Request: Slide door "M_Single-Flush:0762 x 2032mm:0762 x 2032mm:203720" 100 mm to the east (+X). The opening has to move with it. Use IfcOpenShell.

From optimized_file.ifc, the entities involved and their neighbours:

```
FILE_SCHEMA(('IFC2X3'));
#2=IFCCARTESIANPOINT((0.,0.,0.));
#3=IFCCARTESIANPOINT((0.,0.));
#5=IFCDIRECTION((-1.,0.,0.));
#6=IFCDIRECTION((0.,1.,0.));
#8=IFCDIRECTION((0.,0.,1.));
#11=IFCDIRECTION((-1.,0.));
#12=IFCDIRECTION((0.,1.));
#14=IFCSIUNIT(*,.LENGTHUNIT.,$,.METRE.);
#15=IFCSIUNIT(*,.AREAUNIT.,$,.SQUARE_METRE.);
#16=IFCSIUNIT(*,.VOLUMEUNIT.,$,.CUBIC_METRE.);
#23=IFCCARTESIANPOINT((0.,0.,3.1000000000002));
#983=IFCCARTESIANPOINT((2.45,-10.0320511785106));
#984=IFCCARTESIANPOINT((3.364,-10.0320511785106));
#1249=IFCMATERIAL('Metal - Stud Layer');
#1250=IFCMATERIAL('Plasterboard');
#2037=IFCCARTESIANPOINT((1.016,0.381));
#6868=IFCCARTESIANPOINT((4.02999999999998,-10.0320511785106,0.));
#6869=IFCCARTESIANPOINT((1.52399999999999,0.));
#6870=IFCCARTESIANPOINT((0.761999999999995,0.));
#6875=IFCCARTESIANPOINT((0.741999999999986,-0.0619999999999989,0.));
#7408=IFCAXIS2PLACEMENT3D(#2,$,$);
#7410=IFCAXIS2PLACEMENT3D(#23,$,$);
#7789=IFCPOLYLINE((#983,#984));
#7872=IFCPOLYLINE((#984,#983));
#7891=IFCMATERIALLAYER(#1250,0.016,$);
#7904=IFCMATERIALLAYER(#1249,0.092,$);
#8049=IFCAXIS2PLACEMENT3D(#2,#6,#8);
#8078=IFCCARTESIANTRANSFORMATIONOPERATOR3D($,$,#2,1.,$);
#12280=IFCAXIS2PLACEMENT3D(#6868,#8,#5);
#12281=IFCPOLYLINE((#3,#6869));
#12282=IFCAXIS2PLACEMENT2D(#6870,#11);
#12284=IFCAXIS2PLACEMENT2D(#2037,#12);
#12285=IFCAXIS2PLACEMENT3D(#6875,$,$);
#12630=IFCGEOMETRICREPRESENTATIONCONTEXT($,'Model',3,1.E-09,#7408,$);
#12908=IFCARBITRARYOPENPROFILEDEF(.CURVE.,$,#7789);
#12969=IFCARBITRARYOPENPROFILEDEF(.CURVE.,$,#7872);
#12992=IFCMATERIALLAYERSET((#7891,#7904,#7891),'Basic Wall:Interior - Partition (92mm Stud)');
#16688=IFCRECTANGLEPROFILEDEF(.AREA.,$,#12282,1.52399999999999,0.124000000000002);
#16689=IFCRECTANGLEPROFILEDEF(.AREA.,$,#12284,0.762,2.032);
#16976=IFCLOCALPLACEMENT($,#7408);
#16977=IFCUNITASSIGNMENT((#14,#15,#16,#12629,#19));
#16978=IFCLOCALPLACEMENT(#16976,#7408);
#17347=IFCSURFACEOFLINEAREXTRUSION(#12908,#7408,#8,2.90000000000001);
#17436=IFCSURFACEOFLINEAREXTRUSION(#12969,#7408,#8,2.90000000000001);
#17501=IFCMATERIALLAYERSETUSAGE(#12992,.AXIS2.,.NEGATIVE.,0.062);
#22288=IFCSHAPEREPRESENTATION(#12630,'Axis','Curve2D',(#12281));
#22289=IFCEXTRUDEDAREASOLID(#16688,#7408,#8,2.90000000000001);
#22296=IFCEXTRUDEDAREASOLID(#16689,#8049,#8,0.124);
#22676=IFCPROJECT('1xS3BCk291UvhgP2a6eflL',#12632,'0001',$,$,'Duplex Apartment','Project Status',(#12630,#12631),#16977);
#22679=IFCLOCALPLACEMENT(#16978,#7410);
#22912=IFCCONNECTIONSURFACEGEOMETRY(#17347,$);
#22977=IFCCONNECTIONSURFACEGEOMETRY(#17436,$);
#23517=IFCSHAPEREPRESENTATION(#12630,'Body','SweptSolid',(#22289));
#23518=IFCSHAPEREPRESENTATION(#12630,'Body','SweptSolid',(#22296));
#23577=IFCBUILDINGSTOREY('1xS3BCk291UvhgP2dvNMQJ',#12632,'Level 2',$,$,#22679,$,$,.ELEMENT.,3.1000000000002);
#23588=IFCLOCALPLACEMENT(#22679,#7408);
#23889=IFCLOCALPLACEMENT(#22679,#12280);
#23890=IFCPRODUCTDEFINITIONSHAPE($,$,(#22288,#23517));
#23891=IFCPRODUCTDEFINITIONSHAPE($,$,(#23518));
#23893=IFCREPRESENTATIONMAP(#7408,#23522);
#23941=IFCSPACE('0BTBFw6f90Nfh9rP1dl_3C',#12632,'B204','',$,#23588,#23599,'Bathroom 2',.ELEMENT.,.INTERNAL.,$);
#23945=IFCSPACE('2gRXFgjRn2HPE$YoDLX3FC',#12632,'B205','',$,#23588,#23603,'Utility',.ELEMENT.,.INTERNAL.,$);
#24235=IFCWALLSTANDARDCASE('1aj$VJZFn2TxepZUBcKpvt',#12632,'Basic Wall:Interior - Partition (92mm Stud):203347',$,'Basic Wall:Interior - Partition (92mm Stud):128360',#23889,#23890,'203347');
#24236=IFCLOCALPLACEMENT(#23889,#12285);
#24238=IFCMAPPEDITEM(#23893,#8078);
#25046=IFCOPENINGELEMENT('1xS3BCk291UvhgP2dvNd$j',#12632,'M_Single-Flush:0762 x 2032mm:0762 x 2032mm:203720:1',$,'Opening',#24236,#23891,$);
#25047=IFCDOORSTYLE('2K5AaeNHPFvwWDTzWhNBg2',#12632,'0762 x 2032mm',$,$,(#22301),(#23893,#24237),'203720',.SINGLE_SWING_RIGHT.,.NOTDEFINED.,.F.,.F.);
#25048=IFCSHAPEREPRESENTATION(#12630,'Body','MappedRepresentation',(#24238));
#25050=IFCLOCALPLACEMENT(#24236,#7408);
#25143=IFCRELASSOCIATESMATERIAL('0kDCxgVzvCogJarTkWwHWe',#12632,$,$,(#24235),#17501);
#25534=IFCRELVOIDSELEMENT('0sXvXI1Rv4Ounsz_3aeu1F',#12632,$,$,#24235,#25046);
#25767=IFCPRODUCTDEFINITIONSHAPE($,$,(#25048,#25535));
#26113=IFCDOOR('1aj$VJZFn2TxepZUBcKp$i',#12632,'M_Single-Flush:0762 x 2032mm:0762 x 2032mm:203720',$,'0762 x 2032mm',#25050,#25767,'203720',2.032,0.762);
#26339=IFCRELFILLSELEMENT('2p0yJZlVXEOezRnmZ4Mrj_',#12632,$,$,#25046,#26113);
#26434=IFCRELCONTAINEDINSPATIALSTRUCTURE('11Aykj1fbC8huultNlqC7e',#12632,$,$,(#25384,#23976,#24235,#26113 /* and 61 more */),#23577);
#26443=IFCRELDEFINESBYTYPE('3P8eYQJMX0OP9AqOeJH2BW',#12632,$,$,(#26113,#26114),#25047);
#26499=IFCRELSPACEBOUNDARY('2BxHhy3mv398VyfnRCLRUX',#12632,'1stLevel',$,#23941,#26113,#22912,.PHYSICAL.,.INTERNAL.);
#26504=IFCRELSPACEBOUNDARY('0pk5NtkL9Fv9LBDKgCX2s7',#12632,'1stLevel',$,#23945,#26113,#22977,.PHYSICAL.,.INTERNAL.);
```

```python
import numpy as np
import ifcopenshell
import ifcopenshell.api.geometry
import ifcopenshell.util.placement
import ifcopenshell.util.unit

model = ifcopenshell.open("optimized_file.ifc")
unit_scale = ifcopenshell.util.unit.calculate_unit_scale(model)

door = model.by_guid("1aj$VJZFn2TxepZUBcKp$i")
opening = door.FillsVoids[0].RelatingOpeningElement
wall = opening.VoidsElements[0].RelatingBuildingElement

wall_matrix = ifcopenshell.util.placement.get_local_placement(wall.ObjectPlacement)
shift = wall_matrix[:3, 0] * -0.1 / unit_scale
before = ifcopenshell.util.placement.get_local_placement(door.ObjectPlacement)[:3, 3].copy()

# The door is placed relative to its opening, so it follows when the opening moves.
matrix = ifcopenshell.util.placement.get_local_placement(opening.ObjectPlacement)
matrix[:3, 3] += shift
ifcopenshell.api.geometry.edit_object_placement(
    model, product=opening, matrix=matrix, is_si=False, should_transform_children=True
)

# Space boundary surfaces are stored in each space's coordinates; move them too.
for rel in door.ProvidesBoundaries:
    if not rel.ConnectionGeometry:
        continue
    surface = rel.ConnectionGeometry.SurfaceOnRelatingElement
    space_matrix = ifcopenshell.util.placement.get_local_placement(rel.RelatingSpace.ObjectPlacement)
    point = np.array(surface.Position.Location.Coordinates) + space_matrix[:3, :3].T @ shift
    surface.Position = model.createIfcAxis2Placement3D(
        model.createIfcCartesianPoint(point.tolist()), surface.Position.Axis, surface.Position.RefDirection
    )

after = ifcopenshell.util.placement.get_local_placement(door.ObjectPlacement)[:3, 3]
print("door moved by", (after - before).round(3) + 0.0)

model.write("optimized_file_v2.ifc")
```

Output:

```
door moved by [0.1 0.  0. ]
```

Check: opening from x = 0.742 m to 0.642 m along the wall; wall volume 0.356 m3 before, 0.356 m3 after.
